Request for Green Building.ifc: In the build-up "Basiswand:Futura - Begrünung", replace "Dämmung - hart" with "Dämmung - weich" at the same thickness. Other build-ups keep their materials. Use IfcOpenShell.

First a look at what the model holds.

```python
import ifcopenshell
import ifcopenshell.util.element

model = ifcopenshell.open("Green Building.ifc")
print(model.schema)
for layer_set in model.by_type("IfcMaterialLayerSet"):
    if layer_set.LayerSetName == "Basiswand:Futura - Begrünung":
        for layer in layer_set.MaterialLayers:
            print(layer.id(), layer.Material and layer.Material.Name, layer.LayerThickness, sep=" | ")
        print(len(ifcopenshell.util.element.get_elements_by_material(model, layer_set)), "elements and types use it")
print(sorted(m.Name for m in model.by_type("IfcMaterial") if m.Name)[:60])
```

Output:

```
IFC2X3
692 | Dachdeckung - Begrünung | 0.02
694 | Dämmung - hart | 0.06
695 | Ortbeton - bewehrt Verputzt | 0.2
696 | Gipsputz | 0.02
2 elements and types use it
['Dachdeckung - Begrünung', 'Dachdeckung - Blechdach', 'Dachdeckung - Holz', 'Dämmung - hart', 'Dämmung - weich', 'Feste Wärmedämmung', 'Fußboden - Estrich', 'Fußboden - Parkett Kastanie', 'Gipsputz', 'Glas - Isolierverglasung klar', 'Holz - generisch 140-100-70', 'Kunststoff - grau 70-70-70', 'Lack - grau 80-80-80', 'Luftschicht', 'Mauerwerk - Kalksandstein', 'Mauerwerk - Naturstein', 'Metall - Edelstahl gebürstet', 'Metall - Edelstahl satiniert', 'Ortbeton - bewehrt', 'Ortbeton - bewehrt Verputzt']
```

```python
import ifcopenshell
import ifcopenshell.api.material

model = ifcopenshell.open("Green Building.ifc")

layer_set = next(s for s in model.by_type("IfcMaterialLayerSet") if s.LayerSetName == "Basiswand:Futura - Begrünung")
layer = next(l for l in layer_set.MaterialLayers if l.Material and l.Material.Name == "Dämmung - hart")
material = next(m for m in model.by_type("IfcMaterial") if m.Name == "Dämmung - weich")

# Point this one layer at the other material; renaming the old one would change it everywhere.
ifcopenshell.api.material.edit_layer(model, layer=layer, attributes={}, material=material)

print([l.Material.Name if l.Material else None for l in layer_set.MaterialLayers])

model.write("Green Building-out.ifc")
```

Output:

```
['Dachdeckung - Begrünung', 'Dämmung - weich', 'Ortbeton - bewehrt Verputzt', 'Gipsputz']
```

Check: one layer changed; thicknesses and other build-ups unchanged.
